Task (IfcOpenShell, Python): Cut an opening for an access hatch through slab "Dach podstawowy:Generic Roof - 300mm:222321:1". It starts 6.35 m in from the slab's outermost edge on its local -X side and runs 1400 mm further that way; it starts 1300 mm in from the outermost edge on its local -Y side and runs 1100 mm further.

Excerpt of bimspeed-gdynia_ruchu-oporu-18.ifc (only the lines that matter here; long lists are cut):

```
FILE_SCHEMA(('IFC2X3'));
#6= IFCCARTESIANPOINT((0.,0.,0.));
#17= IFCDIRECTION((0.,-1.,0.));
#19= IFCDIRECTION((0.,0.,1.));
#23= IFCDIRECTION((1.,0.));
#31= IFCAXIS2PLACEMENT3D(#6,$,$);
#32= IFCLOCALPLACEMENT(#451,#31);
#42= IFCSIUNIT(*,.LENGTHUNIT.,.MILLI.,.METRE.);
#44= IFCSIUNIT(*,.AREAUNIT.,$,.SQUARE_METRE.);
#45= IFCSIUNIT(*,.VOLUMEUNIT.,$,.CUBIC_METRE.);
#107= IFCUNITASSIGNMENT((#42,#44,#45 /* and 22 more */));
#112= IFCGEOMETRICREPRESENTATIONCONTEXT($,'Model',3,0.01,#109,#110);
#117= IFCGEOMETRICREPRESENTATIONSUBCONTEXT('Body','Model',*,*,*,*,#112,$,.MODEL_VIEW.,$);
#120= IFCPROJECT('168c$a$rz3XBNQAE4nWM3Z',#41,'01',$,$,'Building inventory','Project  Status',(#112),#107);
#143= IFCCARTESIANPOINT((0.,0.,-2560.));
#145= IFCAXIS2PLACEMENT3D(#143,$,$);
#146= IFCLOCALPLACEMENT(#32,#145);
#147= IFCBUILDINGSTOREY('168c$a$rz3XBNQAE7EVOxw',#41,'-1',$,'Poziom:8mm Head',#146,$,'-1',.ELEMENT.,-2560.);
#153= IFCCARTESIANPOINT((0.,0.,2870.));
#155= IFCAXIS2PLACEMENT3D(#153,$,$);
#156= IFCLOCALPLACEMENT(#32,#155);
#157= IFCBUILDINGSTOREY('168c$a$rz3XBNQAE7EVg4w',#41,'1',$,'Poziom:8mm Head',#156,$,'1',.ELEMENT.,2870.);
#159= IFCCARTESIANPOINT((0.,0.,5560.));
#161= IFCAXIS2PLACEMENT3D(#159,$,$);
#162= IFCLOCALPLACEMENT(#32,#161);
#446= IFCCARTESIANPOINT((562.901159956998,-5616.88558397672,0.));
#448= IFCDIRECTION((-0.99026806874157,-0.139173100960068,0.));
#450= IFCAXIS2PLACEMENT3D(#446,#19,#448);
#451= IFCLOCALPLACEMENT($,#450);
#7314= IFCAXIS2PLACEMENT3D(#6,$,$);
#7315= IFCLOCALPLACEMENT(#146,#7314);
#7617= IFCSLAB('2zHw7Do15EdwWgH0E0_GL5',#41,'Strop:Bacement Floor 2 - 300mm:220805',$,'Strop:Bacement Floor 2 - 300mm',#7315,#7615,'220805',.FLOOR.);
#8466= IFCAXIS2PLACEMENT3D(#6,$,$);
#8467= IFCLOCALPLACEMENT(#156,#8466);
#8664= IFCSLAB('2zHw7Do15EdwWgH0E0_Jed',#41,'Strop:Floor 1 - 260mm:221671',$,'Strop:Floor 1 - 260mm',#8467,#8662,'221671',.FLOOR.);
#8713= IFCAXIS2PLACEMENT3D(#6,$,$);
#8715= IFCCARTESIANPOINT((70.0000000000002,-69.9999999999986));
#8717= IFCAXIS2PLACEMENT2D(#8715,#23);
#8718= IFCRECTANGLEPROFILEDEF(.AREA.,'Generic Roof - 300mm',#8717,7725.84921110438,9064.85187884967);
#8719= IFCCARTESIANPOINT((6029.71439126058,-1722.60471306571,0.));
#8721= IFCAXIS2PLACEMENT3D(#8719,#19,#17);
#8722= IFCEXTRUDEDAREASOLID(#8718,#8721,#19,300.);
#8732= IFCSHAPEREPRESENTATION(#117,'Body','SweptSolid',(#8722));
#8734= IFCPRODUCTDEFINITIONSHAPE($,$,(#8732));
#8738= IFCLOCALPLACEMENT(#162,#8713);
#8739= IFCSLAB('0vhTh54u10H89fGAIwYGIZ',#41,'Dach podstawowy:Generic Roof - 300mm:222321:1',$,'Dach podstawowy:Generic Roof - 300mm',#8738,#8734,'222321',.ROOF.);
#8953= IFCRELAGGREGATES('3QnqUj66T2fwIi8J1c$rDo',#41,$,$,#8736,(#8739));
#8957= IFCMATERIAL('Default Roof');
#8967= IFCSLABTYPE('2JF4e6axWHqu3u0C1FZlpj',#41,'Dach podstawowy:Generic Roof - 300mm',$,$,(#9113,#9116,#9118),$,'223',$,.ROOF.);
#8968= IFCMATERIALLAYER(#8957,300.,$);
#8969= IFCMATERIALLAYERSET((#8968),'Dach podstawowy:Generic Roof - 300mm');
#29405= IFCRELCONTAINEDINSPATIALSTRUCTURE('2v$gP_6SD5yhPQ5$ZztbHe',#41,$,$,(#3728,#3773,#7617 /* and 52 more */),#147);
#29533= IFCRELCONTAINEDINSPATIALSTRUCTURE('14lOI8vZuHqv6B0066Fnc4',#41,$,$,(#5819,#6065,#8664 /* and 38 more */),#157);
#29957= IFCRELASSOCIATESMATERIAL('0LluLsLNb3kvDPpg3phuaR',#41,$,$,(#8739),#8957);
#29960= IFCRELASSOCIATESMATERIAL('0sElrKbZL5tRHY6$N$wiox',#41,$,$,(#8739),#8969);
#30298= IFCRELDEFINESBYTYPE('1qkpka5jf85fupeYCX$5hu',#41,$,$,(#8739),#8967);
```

```python
import numpy as np
import ifcopenshell
import ifcopenshell.api.feature
import ifcopenshell.api.geometry
import ifcopenshell.api.root
import ifcopenshell.geom
import ifcopenshell.util.placement
import ifcopenshell.util.representation
import ifcopenshell.util.shape
import ifcopenshell.util.unit

model = ifcopenshell.open("bimspeed-gdynia_ruchu-oporu-18.ifc")
unit_scale = ifcopenshell.util.unit.calculate_unit_scale(model)
settings = ifcopenshell.geom.settings()


def volume(element):
    """Net volume in cubic metres, openings subtracted."""
    shape = ifcopenshell.geom.create_shape(settings, element)
    return ifcopenshell.util.shape.get_volume(shape.geometry)


slab = model.by_guid("0vhTh54u10H89fGAIwYGIZ")
before = volume(slab)

# Extent in the slab's own axes, in metres. The edges named are its -X and -Y sides.
slab_shape = ifcopenshell.geom.create_shape(settings, slab)
vertices = ifcopenshell.util.shape.get_vertices(slab_shape.geometry)
x_min, y_min, bottom = vertices.min(axis=0)
top = vertices[:, 2].max()

opening = ifcopenshell.api.root.create_entity(model, ifc_class="IfcOpeningElement", name="Access hatch opening")
context = ifcopenshell.util.representation.get_context(model, "Model", "Body", "MODEL_VIEW")
width, depth = 1.4, 1.1
outline = [(0.0, 0.0), (width, 0.0), (width, depth), (0.0, depth), (0.0, 0.0)]
# Overshoot both faces by 50 mm so the cut is clean.
shape = ifcopenshell.api.geometry.add_slab_representation(
    model, context=context, depth=top - bottom + 0.1, polyline=outline
)
ifcopenshell.api.geometry.assign_representation(model, product=opening, representation=shape)

matrix = ifcopenshell.util.placement.get_local_placement(slab.ObjectPlacement)
matrix[:, 3] = matrix @ np.append(np.array([x_min + 6.35, y_min + 1.3, bottom - 0.05]) / unit_scale, 1.0)
ifcopenshell.api.geometry.edit_object_placement(model, product=opening, matrix=matrix, is_si=False)
ifcopenshell.api.feature.add_feature(model, feature=opening, element=slab)

after = volume(slab)

print(f"slab volume {before:.3f} -> {after:.3f} m3")

model.write("bimspeed-gdynia_ruchu-oporu-18_rev.ifc")
```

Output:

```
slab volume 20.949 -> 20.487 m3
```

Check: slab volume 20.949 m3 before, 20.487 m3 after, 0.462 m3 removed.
